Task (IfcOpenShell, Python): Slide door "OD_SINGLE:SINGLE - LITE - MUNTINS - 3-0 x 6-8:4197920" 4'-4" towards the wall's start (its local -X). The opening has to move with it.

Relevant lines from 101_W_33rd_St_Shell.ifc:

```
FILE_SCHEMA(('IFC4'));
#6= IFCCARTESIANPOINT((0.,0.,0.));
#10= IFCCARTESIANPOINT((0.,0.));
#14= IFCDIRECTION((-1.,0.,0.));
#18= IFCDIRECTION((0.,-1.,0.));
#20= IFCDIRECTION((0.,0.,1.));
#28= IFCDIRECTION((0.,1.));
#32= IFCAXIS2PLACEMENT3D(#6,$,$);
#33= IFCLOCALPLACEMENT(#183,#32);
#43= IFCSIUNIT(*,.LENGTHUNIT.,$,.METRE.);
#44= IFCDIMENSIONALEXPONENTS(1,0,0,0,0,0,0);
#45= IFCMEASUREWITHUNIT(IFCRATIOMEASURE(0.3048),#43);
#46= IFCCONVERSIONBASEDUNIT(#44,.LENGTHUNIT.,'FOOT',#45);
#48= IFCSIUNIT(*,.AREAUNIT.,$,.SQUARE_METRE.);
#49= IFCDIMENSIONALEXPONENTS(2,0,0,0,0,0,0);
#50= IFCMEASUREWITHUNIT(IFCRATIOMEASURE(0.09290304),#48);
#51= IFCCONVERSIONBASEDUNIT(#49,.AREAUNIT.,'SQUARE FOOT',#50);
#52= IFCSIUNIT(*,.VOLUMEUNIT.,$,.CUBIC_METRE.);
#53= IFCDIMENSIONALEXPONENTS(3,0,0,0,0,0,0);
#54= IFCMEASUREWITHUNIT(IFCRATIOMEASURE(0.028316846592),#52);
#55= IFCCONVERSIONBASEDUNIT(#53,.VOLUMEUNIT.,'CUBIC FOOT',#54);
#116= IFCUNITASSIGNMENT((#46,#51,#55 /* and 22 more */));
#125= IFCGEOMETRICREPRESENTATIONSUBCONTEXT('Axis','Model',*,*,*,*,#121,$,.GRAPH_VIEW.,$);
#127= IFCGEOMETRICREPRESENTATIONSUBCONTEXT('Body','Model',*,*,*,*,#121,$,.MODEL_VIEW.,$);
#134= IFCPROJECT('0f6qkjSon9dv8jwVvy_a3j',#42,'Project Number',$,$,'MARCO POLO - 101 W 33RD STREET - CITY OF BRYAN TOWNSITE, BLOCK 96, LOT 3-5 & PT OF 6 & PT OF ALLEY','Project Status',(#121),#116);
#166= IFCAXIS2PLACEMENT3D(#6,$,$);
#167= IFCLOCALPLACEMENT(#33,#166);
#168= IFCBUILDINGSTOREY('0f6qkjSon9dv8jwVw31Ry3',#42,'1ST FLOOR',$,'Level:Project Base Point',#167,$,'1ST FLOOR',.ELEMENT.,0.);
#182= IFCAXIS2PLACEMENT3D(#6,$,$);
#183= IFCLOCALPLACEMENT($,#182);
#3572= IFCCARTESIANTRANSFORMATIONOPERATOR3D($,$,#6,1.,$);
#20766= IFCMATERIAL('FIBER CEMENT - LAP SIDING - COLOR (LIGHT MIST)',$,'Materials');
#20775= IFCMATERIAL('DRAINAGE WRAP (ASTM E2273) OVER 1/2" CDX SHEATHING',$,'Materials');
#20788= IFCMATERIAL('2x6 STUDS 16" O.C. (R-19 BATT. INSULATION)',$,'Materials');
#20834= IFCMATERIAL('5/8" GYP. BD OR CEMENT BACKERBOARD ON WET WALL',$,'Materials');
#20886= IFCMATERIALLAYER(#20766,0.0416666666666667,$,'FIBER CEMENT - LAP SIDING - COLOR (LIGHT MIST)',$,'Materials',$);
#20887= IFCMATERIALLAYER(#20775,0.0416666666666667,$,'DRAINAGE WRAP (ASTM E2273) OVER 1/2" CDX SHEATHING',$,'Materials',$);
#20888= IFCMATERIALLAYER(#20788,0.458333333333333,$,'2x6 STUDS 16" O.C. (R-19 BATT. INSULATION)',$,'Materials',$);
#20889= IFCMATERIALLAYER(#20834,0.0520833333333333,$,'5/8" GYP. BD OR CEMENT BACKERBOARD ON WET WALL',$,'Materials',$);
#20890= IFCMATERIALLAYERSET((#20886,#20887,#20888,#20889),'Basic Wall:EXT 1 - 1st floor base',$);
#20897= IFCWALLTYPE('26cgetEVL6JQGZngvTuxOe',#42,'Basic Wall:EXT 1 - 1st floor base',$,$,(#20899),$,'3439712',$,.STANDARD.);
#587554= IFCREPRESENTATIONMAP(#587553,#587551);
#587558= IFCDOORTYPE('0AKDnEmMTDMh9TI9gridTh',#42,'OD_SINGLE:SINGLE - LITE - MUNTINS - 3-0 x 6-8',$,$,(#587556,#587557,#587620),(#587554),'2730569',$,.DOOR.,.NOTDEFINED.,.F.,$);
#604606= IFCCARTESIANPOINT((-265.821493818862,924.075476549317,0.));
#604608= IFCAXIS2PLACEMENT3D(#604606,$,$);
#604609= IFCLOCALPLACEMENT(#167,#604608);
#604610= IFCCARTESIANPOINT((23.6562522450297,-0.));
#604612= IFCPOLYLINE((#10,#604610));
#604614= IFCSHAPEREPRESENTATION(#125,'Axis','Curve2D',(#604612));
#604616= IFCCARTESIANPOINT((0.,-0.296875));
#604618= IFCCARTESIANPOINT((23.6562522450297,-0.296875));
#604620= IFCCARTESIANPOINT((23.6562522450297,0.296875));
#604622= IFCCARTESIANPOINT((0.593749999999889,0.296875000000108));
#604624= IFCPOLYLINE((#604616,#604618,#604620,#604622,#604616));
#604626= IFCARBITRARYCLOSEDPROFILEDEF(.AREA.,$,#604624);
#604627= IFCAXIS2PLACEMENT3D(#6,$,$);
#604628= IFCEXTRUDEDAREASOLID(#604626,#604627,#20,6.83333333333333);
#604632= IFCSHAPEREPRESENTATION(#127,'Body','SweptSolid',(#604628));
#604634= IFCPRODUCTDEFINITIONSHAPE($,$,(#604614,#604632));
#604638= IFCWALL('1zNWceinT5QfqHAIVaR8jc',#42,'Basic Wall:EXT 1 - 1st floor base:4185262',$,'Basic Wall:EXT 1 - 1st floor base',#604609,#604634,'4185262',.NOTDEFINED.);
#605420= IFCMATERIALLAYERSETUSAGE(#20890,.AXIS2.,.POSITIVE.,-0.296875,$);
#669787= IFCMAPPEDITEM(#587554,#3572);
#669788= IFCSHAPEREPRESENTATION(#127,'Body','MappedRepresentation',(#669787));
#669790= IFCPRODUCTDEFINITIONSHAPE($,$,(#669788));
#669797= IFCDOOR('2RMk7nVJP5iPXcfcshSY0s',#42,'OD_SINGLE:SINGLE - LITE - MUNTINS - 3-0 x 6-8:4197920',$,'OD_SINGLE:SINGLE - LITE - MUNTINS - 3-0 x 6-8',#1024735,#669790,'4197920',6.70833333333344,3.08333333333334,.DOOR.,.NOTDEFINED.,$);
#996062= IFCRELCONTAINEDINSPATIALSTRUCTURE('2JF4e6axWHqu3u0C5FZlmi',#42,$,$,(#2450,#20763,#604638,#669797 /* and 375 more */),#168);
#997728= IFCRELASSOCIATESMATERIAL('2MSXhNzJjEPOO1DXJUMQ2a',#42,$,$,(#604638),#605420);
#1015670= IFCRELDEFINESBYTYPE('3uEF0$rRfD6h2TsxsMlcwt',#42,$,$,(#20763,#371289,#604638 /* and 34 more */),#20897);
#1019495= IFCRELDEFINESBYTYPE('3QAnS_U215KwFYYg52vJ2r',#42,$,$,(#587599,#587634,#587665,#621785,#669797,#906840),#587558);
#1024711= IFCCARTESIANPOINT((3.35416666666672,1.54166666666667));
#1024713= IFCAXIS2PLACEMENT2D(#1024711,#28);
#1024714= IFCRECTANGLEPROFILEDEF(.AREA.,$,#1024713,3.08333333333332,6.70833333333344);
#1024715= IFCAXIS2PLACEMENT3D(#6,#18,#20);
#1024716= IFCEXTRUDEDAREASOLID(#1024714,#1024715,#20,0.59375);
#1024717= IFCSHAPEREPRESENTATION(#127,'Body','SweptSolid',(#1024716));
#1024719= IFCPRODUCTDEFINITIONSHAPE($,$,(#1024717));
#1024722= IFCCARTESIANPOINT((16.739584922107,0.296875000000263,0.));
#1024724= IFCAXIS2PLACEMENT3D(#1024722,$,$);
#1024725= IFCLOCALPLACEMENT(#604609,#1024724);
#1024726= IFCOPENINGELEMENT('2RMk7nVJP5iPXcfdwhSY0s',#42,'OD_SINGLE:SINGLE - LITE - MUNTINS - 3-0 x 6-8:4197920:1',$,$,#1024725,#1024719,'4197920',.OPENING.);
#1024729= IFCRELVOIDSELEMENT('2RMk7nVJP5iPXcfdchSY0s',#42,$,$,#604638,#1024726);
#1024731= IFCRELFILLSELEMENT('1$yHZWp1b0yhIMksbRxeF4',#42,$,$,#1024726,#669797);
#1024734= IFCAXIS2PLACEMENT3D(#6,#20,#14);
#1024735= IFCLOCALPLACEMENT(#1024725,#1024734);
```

```python
import ifcopenshell
import ifcopenshell.api.geometry
import ifcopenshell.util.placement
import ifcopenshell.util.unit

model = ifcopenshell.open("101_W_33rd_St_Shell.ifc")
unit_scale = ifcopenshell.util.unit.calculate_unit_scale(model)

door = model.by_guid("2RMk7nVJP5iPXcfcshSY0s")
opening = door.FillsVoids[0].RelatingOpeningElement
wall = opening.VoidsElements[0].RelatingBuildingElement

wall_matrix = ifcopenshell.util.placement.get_local_placement(wall.ObjectPlacement)
shift = wall_matrix[:3, 0] * -52 * 0.0254 / unit_scale
before = ifcopenshell.util.placement.get_local_placement(door.ObjectPlacement)[:3, 3].copy()

# The door is placed relative to its opening, so it follows when the opening moves.
matrix = ifcopenshell.util.placement.get_local_placement(opening.ObjectPlacement)
matrix[:3, 3] += shift
ifcopenshell.api.geometry.edit_object_placement(
    model, product=opening, matrix=matrix, is_si=False, should_transform_children=True
)

after = ifcopenshell.util.placement.get_local_placement(door.ObjectPlacement)[:3, 3]
print("door moved by", (after - before).round(3) + 0.0)

model.write("101_W_33rd_St_Shell_v2.ifc")
```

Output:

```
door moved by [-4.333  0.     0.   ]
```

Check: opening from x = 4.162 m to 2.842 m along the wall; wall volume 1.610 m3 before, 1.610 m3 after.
